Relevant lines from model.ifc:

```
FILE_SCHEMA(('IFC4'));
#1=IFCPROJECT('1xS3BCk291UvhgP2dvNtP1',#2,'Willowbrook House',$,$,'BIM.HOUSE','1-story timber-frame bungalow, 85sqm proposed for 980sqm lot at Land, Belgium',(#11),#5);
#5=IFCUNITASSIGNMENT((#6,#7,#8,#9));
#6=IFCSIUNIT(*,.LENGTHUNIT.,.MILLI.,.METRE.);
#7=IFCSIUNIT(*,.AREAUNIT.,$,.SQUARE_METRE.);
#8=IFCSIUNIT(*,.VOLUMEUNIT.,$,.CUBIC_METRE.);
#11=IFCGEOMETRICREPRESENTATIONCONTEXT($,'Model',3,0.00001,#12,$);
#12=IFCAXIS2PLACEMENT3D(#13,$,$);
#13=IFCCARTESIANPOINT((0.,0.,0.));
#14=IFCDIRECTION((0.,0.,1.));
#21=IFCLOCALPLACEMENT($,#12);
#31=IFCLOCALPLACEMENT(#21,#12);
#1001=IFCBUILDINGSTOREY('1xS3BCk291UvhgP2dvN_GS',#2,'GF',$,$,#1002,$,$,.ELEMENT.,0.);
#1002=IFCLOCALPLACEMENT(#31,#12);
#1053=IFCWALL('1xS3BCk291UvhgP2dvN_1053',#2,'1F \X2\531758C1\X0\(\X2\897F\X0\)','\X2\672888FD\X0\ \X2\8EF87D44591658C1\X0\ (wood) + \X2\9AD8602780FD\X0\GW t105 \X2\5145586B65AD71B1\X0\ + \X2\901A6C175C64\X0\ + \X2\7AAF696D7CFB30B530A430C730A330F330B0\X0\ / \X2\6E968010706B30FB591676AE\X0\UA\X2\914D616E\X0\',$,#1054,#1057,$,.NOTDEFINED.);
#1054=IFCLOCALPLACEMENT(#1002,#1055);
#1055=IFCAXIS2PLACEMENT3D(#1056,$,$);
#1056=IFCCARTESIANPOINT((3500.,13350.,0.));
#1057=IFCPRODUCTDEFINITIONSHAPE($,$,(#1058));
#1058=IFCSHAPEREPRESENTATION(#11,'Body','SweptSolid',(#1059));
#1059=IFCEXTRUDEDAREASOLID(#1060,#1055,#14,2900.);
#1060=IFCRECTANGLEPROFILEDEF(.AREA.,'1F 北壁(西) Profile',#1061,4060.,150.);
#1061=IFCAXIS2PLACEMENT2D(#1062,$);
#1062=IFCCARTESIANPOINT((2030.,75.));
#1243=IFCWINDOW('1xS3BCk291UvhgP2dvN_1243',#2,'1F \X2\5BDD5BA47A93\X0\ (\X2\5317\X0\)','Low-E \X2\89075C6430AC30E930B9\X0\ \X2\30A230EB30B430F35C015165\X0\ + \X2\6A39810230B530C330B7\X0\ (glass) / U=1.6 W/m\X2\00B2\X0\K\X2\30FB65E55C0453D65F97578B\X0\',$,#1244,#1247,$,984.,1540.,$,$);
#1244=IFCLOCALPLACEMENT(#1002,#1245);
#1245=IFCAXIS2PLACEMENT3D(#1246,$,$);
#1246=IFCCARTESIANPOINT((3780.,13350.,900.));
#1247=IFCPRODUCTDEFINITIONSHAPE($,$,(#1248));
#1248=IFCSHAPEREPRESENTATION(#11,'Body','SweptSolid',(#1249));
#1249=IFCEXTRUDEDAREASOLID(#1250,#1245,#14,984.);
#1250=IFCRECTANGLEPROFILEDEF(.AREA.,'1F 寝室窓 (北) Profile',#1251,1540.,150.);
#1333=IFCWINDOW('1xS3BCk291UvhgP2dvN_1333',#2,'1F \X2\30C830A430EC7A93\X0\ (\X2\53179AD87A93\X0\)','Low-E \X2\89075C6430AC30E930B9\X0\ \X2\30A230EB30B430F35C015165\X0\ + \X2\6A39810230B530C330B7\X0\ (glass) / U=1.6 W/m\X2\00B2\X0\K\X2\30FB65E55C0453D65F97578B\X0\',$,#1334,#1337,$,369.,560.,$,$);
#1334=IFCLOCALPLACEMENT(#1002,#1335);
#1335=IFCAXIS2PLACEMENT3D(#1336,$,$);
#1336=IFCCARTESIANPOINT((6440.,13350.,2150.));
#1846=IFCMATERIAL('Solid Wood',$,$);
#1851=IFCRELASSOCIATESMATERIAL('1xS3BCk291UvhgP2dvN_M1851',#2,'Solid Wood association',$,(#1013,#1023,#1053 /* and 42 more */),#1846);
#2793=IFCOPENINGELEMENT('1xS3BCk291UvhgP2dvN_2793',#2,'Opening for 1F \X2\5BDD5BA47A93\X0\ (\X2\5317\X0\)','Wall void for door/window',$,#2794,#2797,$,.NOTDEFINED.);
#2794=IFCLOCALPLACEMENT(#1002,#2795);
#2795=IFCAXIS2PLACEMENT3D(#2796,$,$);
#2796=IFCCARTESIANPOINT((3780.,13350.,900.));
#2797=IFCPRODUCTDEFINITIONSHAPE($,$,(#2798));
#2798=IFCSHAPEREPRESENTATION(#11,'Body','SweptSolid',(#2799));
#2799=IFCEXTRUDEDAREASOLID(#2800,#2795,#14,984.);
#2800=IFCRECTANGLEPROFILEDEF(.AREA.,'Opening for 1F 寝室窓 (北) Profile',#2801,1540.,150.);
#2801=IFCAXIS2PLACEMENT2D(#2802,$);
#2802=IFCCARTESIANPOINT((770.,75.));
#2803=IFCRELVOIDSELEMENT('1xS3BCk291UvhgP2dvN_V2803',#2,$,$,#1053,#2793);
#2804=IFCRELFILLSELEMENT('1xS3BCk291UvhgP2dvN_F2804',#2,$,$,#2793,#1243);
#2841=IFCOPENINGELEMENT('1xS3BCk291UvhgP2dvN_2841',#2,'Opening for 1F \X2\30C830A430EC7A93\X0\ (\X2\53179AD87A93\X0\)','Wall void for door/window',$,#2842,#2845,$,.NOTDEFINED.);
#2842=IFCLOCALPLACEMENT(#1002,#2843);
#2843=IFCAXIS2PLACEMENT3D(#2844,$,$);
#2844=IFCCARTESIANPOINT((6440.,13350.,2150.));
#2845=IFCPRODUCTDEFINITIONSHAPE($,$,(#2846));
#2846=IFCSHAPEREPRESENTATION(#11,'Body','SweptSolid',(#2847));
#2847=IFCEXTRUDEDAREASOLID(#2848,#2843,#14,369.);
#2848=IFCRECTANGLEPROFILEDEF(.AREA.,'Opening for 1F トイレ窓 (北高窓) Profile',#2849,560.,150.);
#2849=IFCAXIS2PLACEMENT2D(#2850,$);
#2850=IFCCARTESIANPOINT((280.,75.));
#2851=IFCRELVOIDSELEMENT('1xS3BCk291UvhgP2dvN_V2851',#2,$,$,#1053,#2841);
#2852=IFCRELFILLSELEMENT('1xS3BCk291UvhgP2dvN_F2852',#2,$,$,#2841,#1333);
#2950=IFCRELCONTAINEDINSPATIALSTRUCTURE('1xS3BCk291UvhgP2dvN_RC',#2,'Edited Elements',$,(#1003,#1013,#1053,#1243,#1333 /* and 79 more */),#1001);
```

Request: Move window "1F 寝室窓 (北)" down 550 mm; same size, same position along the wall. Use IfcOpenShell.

```python
import numpy as np
import ifcopenshell
import ifcopenshell.api.geometry
import ifcopenshell.util.placement
import ifcopenshell.util.unit

model = ifcopenshell.open("model.ifc")
unit_scale = ifcopenshell.util.unit.calculate_unit_scale(model)

window = model.by_guid("1xS3BCk291UvhgP2dvN_1243")
opening = window.FillsVoids[0].RelatingOpeningElement
dz = -550.0

shift = np.array([0.0, 0.0, dz])
# The window is not placed relative to its opening, so move both.
for product in (opening, window):
    matrix = ifcopenshell.util.placement.get_local_placement(product.ObjectPlacement)
    matrix[:3, 3] += shift
    ifcopenshell.api.geometry.edit_object_placement(model, product=product, matrix=matrix, is_si=False)

print(f"moved by {dz * unit_scale:+.3f} m")

model.write("model_updated.ifc")
```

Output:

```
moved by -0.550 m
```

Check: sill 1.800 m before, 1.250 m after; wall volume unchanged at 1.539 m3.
